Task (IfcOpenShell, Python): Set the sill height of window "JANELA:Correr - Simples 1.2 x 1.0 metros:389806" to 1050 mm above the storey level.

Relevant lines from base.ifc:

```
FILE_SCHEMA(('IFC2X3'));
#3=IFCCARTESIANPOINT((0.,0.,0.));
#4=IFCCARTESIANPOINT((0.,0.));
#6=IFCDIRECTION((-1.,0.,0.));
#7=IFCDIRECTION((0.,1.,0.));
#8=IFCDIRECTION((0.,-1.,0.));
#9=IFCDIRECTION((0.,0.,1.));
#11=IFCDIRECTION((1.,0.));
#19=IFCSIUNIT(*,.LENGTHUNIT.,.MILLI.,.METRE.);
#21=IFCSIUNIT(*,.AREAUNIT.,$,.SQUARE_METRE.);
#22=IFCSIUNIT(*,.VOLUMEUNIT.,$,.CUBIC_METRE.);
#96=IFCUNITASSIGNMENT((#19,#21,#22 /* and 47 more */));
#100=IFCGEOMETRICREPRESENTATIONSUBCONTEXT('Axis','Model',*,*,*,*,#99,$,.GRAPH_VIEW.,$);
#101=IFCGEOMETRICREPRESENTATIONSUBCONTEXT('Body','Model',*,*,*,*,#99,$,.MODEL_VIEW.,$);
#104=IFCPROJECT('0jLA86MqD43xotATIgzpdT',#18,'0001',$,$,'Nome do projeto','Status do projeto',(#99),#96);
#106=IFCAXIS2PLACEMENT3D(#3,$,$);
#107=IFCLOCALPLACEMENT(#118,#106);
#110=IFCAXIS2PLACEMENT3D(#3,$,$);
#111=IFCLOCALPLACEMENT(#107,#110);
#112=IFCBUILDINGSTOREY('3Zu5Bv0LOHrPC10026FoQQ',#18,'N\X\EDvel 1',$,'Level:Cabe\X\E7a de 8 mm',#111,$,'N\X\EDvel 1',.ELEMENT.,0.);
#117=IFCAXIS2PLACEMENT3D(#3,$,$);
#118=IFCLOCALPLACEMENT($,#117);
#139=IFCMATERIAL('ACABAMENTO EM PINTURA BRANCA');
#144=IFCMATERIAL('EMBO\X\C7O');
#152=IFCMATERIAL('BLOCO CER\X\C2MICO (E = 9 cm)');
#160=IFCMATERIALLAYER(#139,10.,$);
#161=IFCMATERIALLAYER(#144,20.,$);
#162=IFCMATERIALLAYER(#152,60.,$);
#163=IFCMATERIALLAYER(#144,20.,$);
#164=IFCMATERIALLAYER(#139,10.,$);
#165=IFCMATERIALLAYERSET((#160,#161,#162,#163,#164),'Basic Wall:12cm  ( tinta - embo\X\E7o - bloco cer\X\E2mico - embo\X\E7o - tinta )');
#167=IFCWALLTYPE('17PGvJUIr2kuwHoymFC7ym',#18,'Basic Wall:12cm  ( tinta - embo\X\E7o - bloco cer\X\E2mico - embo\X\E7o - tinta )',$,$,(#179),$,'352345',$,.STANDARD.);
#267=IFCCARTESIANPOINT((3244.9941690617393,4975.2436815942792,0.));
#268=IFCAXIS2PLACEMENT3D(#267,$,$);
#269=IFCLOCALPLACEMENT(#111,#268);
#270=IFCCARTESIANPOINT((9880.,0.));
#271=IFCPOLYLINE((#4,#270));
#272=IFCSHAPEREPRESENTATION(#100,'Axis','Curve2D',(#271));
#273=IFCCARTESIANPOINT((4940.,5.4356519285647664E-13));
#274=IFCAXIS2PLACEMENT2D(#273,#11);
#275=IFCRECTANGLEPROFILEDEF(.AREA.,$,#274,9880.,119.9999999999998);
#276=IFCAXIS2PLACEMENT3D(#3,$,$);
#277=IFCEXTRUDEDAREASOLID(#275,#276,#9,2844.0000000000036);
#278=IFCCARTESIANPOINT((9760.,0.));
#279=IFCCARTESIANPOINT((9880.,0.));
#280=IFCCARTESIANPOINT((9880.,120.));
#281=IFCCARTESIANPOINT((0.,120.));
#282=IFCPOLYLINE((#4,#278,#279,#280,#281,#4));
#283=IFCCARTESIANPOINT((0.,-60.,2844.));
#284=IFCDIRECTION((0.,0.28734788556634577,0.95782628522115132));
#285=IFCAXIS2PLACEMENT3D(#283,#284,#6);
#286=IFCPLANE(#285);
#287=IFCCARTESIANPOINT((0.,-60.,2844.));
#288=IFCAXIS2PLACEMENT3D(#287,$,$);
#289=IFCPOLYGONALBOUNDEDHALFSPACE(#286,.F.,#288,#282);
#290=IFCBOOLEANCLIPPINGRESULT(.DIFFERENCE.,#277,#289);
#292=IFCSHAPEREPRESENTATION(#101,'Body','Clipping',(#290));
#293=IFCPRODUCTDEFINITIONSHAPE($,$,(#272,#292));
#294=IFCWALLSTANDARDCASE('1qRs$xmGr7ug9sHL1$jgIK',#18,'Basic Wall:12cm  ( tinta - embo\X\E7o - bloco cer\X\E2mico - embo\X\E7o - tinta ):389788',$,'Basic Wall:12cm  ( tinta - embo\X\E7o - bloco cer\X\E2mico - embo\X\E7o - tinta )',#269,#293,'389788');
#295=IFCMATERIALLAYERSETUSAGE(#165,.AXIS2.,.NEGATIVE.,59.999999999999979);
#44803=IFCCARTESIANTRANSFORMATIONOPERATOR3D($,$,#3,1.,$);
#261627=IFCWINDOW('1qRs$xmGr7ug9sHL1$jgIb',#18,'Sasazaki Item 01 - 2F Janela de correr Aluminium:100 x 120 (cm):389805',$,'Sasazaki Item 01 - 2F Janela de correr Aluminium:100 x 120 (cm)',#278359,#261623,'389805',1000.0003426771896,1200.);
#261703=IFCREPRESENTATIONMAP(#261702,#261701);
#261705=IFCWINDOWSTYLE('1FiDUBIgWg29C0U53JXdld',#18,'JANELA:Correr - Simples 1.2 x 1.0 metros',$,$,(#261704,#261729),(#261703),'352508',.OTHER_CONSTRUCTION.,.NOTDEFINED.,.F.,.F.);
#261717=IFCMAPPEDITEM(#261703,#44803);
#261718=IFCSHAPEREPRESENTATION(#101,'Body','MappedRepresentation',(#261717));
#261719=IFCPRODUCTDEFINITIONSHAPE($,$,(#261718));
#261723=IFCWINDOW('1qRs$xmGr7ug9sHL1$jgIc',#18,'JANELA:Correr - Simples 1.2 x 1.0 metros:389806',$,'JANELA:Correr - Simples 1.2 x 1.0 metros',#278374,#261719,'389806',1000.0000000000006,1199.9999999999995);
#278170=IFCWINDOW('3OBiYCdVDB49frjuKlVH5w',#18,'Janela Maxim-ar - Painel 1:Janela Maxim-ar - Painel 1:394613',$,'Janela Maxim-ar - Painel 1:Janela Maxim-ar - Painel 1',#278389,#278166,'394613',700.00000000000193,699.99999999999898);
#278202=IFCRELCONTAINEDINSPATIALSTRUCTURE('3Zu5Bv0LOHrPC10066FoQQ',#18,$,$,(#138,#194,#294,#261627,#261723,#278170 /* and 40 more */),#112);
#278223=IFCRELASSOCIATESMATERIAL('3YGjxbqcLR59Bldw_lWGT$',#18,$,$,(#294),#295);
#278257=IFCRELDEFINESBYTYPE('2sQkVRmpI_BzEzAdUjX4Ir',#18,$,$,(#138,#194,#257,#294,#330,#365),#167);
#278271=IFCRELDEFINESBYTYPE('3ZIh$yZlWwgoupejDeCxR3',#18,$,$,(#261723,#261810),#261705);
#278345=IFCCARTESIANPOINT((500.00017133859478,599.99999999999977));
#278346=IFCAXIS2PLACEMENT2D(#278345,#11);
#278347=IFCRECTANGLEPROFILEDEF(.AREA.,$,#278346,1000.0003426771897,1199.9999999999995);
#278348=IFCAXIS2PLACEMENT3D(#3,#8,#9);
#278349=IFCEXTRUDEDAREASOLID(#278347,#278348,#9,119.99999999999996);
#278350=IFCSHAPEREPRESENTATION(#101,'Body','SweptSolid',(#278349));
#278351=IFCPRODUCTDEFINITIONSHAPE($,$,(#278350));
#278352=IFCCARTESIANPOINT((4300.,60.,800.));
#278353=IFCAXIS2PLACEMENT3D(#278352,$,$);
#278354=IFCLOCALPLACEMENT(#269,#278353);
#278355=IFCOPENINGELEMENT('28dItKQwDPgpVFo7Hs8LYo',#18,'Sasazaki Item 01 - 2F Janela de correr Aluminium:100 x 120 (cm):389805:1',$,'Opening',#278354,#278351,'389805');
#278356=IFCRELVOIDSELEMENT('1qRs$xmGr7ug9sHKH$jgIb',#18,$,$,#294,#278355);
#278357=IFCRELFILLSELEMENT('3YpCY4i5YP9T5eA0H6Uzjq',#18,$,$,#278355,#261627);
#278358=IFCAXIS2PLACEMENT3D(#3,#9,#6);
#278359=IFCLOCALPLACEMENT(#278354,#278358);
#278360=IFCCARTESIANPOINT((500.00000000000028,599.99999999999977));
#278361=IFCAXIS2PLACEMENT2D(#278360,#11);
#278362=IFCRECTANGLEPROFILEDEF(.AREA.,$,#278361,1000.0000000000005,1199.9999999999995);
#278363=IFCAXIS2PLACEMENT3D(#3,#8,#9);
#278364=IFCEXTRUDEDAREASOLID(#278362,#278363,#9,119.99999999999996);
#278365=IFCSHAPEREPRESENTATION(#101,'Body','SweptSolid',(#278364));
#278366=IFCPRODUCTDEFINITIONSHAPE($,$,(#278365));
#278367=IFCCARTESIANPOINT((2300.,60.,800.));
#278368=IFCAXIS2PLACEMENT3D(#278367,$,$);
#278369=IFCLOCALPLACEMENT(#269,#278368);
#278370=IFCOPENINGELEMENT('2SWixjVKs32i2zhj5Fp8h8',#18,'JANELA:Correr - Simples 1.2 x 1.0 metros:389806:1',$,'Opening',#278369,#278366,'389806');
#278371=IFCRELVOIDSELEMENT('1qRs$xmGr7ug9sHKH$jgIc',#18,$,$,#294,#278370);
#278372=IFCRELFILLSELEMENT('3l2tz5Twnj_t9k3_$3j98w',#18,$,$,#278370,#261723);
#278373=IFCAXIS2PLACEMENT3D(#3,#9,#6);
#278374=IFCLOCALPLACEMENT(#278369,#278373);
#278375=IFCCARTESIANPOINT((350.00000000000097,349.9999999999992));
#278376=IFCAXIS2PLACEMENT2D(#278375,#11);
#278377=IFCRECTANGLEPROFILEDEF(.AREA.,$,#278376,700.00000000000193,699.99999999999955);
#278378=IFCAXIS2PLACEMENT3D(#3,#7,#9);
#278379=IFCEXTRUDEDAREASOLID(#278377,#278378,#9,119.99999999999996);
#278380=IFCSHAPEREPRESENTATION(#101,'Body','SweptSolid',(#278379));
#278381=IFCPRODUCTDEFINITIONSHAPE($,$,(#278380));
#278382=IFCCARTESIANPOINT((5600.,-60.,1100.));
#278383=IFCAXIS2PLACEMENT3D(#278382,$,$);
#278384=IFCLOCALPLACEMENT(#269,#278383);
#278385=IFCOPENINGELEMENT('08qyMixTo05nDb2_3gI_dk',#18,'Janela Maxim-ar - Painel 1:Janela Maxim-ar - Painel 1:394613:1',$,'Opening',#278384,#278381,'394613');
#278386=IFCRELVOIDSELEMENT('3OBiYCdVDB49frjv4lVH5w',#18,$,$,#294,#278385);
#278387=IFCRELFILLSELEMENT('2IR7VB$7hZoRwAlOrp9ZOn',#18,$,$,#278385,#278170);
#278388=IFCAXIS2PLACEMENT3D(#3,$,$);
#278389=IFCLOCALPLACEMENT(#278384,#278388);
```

```python
import numpy as np
import ifcopenshell
import ifcopenshell.api.geometry
import ifcopenshell.geom
import ifcopenshell.util.element
import ifcopenshell.util.placement
import ifcopenshell.util.shape
import ifcopenshell.util.unit

model = ifcopenshell.open("base.ifc")
unit_scale = ifcopenshell.util.unit.calculate_unit_scale(model)

window = model.by_guid("1qRs$xmGr7ug9sHL1$jgIc")
opening = window.FillsVoids[0].RelatingOpeningElement
storey = ifcopenshell.util.element.get_container(window, ifc_class="IfcBuildingStorey")
level = ifcopenshell.util.placement.get_local_placement(storey.ObjectPlacement)[2, 3]

# The opening's origin need not be at the sill, so measure its lowest point.
shape = ifcopenshell.geom.create_shape(ifcopenshell.geom.settings(), opening)
bottom = ifcopenshell.util.shape.get_shape_bottom_elevation(shape, shape.geometry) / unit_scale
dz = level + 1.05 / unit_scale - bottom

shift = np.array([0.0, 0.0, dz])
# The window is placed relative to its opening, so it follows when the opening moves.
matrix = ifcopenshell.util.placement.get_local_placement(opening.ObjectPlacement)
matrix[:3, 3] += shift
ifcopenshell.api.geometry.edit_object_placement(
    model, product=opening, matrix=matrix, is_si=False, should_transform_children=True
)

print(f"moved by {dz * unit_scale:+.3f} m")

model.write("base_rev.ifc")
```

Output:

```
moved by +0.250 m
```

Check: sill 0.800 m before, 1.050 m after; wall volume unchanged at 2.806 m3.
